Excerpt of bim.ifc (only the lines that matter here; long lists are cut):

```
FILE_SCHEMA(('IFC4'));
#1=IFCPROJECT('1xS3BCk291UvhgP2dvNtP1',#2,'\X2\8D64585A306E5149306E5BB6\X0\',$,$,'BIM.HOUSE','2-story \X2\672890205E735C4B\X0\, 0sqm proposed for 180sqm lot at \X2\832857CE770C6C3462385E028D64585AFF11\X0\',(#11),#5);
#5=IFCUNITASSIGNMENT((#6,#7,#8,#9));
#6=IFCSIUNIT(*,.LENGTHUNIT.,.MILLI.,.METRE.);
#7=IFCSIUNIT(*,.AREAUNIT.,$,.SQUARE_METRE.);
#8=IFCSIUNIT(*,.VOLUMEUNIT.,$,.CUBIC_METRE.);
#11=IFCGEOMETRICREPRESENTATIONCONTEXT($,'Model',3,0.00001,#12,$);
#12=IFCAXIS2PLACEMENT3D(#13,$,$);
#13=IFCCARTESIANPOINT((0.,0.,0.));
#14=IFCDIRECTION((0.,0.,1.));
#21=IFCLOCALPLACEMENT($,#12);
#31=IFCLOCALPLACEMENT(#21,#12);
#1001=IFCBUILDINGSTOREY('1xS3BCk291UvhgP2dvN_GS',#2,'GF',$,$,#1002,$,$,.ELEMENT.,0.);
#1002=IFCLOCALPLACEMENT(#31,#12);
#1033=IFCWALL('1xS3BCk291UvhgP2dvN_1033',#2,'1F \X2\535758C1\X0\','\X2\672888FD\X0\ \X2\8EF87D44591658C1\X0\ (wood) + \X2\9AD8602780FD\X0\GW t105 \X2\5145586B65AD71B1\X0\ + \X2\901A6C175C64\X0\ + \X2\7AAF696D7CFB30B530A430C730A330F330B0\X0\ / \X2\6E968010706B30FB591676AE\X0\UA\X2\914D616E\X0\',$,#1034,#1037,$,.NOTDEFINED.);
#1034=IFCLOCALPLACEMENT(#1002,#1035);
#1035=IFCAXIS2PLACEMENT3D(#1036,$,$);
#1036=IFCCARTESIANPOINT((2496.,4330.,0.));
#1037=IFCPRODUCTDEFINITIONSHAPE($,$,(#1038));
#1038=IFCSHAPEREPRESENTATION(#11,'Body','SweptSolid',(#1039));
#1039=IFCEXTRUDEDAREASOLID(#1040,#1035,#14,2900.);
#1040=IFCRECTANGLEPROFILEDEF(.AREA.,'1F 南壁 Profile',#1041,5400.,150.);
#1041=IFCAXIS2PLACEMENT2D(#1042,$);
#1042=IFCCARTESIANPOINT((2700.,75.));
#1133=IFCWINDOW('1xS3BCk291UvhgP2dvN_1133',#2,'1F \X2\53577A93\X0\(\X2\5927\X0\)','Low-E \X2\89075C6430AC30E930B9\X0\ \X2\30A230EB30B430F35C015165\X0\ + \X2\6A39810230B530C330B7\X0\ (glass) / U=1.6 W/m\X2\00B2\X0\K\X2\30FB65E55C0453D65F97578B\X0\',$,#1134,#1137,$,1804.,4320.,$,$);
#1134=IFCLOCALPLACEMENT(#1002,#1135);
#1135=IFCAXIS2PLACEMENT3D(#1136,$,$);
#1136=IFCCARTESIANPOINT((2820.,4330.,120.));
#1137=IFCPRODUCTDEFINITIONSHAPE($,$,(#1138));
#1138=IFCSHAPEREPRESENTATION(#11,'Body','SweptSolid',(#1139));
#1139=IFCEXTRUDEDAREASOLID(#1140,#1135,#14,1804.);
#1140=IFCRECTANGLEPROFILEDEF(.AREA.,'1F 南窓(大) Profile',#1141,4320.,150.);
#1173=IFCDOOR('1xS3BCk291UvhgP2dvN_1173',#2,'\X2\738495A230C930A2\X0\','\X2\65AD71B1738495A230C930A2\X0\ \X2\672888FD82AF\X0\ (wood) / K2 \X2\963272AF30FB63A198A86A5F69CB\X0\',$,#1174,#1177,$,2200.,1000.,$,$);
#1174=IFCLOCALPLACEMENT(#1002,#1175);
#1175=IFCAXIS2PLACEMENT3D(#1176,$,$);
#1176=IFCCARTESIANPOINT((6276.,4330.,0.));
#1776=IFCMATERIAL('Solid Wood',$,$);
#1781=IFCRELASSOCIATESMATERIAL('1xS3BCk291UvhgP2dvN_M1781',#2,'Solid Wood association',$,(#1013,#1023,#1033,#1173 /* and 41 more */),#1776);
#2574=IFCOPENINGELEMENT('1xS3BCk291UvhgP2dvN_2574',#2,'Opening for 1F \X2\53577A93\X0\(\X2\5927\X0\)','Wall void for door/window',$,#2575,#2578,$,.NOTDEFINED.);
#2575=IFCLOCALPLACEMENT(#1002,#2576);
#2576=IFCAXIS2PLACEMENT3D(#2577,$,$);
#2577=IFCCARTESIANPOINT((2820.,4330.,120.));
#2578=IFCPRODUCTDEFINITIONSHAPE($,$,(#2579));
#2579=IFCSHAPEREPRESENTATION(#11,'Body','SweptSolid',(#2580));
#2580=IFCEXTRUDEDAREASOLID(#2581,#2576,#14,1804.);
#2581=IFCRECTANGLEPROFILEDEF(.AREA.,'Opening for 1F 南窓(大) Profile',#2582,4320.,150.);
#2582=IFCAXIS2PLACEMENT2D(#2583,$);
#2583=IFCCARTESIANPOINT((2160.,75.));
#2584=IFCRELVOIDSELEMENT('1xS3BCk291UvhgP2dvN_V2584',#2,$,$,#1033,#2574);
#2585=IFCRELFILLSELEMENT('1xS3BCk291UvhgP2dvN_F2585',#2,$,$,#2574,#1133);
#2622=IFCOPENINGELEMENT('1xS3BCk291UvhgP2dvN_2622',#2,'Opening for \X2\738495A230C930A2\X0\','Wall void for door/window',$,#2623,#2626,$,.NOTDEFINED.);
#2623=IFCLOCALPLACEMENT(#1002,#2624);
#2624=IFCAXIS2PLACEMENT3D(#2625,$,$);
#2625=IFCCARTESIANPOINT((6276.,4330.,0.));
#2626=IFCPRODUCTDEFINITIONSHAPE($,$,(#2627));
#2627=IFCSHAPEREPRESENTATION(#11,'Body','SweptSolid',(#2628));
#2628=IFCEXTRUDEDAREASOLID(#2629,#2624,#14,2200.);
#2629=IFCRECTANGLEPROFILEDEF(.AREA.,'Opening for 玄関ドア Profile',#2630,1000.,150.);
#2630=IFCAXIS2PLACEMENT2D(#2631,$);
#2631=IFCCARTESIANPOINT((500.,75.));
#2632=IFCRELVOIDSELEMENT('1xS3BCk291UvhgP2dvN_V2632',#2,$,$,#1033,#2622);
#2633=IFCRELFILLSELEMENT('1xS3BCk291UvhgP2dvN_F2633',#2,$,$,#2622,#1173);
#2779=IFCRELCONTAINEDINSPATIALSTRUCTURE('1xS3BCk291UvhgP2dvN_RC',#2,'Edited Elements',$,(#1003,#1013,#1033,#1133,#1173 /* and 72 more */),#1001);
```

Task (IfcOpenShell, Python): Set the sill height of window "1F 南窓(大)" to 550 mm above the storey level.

```python
import numpy as np
import ifcopenshell
import ifcopenshell.api.geometry
import ifcopenshell.geom
import ifcopenshell.util.element
import ifcopenshell.util.placement
import ifcopenshell.util.shape
import ifcopenshell.util.unit

model = ifcopenshell.open("bim.ifc")
unit_scale = ifcopenshell.util.unit.calculate_unit_scale(model)

window = model.by_guid("1xS3BCk291UvhgP2dvN_1133")
opening = window.FillsVoids[0].RelatingOpeningElement
storey = ifcopenshell.util.element.get_container(window, ifc_class="IfcBuildingStorey")
level = ifcopenshell.util.placement.get_local_placement(storey.ObjectPlacement)[2, 3]

# The opening's origin need not be at the sill, so measure its lowest point.
shape = ifcopenshell.geom.create_shape(ifcopenshell.geom.settings(), opening)
bottom = ifcopenshell.util.shape.get_shape_bottom_elevation(shape, shape.geometry) / unit_scale
dz = level + 0.55 / unit_scale - bottom

shift = np.array([0.0, 0.0, dz])
# The window is not placed relative to its opening, so move both.
for product in (opening, window):
    matrix = ifcopenshell.util.placement.get_local_placement(product.ObjectPlacement)
    matrix[:3, 3] += shift
    ifcopenshell.api.geometry.edit_object_placement(model, product=product, matrix=matrix, is_si=False)

print(f"moved by {dz * unit_scale:+.3f} m")

model.write("bim-out.ifc")
```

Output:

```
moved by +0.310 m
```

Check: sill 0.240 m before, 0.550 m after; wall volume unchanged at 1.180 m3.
